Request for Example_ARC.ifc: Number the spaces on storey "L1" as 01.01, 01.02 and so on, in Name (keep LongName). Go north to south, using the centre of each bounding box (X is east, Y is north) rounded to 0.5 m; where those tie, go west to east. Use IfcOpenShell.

First a look at what the model holds.

```python
import ifcopenshell
import ifcopenshell.util.element
import ifcopenshell.util.placement

model = ifcopenshell.open("Example_ARC.ifc")
print(model.schema)
storey = next(s for s in model.by_type("IfcBuildingStorey") if s.Name == "L1")
spaces = [e for e in ifcopenshell.util.element.get_decomposition(storey) if e.is_a("IfcSpace")]
for e in sorted(spaces, key=lambda e: e.id()):
    origin = ifcopenshell.util.placement.get_local_placement(e.ObjectPlacement)[:3, 3]
    print(e.id(), e.Name, e.LongName, origin.round(2) + 0.0, sep=" | ")
```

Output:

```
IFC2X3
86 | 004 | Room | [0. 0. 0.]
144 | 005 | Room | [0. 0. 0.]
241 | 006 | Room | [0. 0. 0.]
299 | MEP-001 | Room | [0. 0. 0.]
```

```python
import ifcopenshell
import ifcopenshell.geom
import ifcopenshell.util.element
import ifcopenshell.util.shape

model = ifcopenshell.open("Example_ARC.ifc")
settings = ifcopenshell.geom.settings()
settings.set("use-world-coords", True)


def centre(element):
    shape = ifcopenshell.geom.create_shape(settings, element)
    return ifcopenshell.util.shape.get_bbox_centroid(shape.geometry)


storey = next(s for s in model.by_type("IfcBuildingStorey") if s.Name == "L1")
spaces = [e for e in ifcopenshell.util.element.get_decomposition(storey) if e.is_a("IfcSpace")]

# Insertion points can sit at a corner or the storey origin, so sort by the geometry (in metres).
centres = {e: centre(e) for e in spaces}
spaces.sort(key=lambda e: (-round(centres[e][1] / 0.5), centres[e][0]))

for i, e in enumerate(spaces, start=1):
    number = f"01.{i:02d}"
    e.Name = number
    print(e.id(), number)

model.write("Example_ARC_v2.ifc")
```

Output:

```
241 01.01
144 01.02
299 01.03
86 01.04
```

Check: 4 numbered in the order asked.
